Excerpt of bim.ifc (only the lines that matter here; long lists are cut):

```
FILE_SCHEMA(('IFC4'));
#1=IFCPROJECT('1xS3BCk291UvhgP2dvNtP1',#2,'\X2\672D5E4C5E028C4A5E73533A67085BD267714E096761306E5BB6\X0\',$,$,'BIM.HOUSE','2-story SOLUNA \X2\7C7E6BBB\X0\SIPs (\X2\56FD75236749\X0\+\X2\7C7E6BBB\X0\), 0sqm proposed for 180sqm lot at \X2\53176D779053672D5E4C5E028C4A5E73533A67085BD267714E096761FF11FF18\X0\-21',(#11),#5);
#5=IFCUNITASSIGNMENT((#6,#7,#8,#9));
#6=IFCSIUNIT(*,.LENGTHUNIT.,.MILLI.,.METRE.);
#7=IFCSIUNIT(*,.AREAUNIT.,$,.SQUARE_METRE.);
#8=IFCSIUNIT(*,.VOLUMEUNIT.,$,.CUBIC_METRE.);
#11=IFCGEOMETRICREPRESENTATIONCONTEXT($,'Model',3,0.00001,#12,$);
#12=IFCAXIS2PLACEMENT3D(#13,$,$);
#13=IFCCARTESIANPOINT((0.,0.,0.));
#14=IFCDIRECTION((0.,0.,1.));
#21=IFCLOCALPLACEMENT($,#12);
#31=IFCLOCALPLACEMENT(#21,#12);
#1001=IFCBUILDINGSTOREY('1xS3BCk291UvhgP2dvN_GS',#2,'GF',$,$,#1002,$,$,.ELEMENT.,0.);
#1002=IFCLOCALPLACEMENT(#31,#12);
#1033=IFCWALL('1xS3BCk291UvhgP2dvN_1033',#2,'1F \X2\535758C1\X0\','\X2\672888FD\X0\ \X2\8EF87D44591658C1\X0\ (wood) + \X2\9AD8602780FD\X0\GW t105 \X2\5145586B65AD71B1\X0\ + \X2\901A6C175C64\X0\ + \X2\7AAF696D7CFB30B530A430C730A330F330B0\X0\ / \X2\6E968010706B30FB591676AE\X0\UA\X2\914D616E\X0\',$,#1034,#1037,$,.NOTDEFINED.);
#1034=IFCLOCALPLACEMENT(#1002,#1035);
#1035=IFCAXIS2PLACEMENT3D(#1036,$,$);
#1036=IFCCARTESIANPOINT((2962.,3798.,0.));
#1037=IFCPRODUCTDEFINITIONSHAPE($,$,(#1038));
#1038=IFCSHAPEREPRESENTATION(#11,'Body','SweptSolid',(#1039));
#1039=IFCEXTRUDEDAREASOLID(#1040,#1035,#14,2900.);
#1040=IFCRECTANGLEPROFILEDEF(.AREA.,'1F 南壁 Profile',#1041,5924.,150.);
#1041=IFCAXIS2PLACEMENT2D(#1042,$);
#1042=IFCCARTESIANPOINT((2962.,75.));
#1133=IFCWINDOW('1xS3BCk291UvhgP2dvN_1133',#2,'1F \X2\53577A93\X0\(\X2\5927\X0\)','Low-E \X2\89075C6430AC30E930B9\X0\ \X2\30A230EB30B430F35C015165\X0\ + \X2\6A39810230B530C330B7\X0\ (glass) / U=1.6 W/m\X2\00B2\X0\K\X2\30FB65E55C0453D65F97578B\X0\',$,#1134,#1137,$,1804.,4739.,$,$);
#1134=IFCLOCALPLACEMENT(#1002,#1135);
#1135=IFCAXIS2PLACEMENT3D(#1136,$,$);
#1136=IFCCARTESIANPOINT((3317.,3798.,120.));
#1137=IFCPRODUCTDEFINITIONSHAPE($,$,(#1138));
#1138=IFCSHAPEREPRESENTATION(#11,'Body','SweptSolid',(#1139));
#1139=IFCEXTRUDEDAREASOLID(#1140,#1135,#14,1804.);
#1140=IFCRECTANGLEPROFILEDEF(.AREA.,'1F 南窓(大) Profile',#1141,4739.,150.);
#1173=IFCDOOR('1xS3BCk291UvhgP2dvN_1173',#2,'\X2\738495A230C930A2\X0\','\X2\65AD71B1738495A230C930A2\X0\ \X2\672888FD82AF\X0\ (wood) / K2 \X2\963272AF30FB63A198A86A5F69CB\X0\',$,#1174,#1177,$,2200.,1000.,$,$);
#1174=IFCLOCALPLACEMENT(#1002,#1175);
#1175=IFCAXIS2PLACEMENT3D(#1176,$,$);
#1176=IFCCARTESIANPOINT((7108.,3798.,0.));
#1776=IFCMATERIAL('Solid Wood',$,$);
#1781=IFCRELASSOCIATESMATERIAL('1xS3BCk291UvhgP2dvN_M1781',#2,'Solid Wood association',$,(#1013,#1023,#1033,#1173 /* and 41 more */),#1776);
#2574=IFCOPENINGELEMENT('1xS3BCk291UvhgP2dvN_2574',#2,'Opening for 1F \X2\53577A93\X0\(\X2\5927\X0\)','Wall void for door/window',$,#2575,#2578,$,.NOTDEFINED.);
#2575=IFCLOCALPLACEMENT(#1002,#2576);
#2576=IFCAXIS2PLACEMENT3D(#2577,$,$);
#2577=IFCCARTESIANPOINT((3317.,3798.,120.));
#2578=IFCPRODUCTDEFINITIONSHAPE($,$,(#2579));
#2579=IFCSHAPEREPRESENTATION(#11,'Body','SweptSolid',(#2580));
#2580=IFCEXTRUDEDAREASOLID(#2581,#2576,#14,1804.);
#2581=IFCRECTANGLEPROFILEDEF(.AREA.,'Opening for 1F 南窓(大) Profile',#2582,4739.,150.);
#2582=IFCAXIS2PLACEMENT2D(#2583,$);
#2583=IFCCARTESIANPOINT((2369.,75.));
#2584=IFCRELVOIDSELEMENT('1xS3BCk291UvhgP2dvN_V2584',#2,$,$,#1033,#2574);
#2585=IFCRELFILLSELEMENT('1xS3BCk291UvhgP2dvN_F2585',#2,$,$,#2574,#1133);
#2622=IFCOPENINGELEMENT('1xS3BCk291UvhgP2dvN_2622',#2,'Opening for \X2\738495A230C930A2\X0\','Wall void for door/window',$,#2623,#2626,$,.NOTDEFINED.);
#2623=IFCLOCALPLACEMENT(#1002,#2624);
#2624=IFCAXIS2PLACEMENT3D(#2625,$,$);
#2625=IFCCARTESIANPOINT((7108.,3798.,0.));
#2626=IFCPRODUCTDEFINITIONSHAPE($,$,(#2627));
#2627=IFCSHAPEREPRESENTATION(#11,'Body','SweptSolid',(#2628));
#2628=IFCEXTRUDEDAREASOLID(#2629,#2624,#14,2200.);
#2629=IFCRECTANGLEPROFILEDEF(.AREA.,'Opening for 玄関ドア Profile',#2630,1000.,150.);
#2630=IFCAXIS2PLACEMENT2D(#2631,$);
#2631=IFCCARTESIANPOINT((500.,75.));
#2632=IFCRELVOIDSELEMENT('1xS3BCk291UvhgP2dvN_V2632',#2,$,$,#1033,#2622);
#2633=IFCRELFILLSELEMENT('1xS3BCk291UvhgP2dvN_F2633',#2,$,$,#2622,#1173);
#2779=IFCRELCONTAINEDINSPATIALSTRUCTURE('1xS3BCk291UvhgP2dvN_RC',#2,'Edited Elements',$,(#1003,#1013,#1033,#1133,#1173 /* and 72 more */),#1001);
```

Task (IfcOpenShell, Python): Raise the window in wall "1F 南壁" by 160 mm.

```python
import numpy as np
import ifcopenshell
import ifcopenshell.api.geometry
import ifcopenshell.util.placement
import ifcopenshell.util.unit

model = ifcopenshell.open("bim.ifc")
unit_scale = ifcopenshell.util.unit.calculate_unit_scale(model)

window = model.by_guid("1xS3BCk291UvhgP2dvN_1133")
opening = window.FillsVoids[0].RelatingOpeningElement
dz = 0.16 / unit_scale

shift = np.array([0.0, 0.0, dz])
# The window is not placed relative to its opening, so move both.
for product in (opening, window):
    matrix = ifcopenshell.util.placement.get_local_placement(product.ObjectPlacement)
    matrix[:3, 3] += shift
    ifcopenshell.api.geometry.edit_object_placement(model, product=product, matrix=matrix, is_si=False)

print(f"moved by {dz * unit_scale:+.3f} m")

model.write("bim_rev.ifc")
```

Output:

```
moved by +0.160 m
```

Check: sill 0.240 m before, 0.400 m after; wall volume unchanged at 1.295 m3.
